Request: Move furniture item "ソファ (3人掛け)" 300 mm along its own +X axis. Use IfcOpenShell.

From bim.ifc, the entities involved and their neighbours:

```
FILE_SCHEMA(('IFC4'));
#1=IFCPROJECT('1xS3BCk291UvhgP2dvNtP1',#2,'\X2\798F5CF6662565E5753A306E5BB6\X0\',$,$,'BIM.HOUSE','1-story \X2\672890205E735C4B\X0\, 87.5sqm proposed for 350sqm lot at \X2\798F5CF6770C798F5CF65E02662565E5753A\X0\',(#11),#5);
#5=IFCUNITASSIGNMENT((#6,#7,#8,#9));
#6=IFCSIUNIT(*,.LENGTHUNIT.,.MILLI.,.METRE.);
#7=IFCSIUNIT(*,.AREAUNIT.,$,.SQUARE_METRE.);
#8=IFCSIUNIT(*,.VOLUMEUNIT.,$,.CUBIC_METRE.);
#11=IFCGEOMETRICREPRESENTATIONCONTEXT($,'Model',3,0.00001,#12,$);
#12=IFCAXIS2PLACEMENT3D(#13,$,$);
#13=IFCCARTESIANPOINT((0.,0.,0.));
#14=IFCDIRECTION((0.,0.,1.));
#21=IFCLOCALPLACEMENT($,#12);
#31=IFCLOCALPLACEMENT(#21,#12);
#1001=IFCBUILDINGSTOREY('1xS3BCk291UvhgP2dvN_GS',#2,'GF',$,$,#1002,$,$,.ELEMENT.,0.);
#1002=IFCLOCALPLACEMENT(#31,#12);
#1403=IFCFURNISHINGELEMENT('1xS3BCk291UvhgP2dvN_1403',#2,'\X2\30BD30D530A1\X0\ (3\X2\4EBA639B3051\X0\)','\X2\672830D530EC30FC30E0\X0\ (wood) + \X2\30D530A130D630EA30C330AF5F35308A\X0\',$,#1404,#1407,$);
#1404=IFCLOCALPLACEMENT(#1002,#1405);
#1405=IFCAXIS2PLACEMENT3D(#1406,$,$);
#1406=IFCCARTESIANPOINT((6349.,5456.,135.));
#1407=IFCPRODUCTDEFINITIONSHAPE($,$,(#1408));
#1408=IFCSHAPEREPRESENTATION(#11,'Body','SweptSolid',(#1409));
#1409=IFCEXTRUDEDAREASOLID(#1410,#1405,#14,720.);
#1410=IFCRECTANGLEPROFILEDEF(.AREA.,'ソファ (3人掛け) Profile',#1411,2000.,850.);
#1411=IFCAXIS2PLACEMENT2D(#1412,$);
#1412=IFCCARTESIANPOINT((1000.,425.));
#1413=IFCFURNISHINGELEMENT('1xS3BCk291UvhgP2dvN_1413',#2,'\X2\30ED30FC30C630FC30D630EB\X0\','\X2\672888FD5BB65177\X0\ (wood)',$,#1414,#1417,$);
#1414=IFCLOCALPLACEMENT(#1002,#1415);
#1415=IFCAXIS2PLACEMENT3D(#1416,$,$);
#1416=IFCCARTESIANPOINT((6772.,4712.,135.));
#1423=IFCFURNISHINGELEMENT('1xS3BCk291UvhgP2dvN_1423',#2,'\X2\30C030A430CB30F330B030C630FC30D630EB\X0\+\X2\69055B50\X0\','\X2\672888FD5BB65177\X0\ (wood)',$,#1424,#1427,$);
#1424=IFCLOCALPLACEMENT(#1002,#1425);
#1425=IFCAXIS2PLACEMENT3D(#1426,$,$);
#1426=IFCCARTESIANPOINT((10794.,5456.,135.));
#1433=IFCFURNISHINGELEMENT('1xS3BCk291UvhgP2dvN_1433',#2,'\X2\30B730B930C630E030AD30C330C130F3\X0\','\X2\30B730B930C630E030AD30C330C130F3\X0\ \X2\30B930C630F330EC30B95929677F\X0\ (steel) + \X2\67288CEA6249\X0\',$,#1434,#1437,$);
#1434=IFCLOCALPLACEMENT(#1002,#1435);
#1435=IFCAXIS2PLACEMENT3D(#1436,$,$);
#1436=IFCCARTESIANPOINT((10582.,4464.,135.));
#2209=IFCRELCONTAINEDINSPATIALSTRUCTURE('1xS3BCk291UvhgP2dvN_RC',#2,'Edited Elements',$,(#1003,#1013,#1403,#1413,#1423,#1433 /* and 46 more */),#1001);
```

```python
import ifcopenshell
import ifcopenshell.api.geometry
import ifcopenshell.util.placement

model = ifcopenshell.open("bim.ifc")

item = model.by_guid("1xS3BCk291UvhgP2dvN_1403")
matrix = ifcopenshell.util.placement.get_local_placement(item.ObjectPlacement)
matrix[:3, 3] += matrix[:3, 0] * 300.0
ifcopenshell.api.geometry.edit_object_placement(model, product=item, matrix=matrix, is_si=False)

print(ifcopenshell.util.placement.get_local_placement(item.ObjectPlacement).round(3) + 0.0)

model.write("bim_edited.ifc")
```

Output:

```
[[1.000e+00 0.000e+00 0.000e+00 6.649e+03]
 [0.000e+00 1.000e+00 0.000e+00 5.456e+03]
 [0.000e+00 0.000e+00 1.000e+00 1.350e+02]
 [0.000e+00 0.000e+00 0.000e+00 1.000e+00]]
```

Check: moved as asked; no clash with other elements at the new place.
